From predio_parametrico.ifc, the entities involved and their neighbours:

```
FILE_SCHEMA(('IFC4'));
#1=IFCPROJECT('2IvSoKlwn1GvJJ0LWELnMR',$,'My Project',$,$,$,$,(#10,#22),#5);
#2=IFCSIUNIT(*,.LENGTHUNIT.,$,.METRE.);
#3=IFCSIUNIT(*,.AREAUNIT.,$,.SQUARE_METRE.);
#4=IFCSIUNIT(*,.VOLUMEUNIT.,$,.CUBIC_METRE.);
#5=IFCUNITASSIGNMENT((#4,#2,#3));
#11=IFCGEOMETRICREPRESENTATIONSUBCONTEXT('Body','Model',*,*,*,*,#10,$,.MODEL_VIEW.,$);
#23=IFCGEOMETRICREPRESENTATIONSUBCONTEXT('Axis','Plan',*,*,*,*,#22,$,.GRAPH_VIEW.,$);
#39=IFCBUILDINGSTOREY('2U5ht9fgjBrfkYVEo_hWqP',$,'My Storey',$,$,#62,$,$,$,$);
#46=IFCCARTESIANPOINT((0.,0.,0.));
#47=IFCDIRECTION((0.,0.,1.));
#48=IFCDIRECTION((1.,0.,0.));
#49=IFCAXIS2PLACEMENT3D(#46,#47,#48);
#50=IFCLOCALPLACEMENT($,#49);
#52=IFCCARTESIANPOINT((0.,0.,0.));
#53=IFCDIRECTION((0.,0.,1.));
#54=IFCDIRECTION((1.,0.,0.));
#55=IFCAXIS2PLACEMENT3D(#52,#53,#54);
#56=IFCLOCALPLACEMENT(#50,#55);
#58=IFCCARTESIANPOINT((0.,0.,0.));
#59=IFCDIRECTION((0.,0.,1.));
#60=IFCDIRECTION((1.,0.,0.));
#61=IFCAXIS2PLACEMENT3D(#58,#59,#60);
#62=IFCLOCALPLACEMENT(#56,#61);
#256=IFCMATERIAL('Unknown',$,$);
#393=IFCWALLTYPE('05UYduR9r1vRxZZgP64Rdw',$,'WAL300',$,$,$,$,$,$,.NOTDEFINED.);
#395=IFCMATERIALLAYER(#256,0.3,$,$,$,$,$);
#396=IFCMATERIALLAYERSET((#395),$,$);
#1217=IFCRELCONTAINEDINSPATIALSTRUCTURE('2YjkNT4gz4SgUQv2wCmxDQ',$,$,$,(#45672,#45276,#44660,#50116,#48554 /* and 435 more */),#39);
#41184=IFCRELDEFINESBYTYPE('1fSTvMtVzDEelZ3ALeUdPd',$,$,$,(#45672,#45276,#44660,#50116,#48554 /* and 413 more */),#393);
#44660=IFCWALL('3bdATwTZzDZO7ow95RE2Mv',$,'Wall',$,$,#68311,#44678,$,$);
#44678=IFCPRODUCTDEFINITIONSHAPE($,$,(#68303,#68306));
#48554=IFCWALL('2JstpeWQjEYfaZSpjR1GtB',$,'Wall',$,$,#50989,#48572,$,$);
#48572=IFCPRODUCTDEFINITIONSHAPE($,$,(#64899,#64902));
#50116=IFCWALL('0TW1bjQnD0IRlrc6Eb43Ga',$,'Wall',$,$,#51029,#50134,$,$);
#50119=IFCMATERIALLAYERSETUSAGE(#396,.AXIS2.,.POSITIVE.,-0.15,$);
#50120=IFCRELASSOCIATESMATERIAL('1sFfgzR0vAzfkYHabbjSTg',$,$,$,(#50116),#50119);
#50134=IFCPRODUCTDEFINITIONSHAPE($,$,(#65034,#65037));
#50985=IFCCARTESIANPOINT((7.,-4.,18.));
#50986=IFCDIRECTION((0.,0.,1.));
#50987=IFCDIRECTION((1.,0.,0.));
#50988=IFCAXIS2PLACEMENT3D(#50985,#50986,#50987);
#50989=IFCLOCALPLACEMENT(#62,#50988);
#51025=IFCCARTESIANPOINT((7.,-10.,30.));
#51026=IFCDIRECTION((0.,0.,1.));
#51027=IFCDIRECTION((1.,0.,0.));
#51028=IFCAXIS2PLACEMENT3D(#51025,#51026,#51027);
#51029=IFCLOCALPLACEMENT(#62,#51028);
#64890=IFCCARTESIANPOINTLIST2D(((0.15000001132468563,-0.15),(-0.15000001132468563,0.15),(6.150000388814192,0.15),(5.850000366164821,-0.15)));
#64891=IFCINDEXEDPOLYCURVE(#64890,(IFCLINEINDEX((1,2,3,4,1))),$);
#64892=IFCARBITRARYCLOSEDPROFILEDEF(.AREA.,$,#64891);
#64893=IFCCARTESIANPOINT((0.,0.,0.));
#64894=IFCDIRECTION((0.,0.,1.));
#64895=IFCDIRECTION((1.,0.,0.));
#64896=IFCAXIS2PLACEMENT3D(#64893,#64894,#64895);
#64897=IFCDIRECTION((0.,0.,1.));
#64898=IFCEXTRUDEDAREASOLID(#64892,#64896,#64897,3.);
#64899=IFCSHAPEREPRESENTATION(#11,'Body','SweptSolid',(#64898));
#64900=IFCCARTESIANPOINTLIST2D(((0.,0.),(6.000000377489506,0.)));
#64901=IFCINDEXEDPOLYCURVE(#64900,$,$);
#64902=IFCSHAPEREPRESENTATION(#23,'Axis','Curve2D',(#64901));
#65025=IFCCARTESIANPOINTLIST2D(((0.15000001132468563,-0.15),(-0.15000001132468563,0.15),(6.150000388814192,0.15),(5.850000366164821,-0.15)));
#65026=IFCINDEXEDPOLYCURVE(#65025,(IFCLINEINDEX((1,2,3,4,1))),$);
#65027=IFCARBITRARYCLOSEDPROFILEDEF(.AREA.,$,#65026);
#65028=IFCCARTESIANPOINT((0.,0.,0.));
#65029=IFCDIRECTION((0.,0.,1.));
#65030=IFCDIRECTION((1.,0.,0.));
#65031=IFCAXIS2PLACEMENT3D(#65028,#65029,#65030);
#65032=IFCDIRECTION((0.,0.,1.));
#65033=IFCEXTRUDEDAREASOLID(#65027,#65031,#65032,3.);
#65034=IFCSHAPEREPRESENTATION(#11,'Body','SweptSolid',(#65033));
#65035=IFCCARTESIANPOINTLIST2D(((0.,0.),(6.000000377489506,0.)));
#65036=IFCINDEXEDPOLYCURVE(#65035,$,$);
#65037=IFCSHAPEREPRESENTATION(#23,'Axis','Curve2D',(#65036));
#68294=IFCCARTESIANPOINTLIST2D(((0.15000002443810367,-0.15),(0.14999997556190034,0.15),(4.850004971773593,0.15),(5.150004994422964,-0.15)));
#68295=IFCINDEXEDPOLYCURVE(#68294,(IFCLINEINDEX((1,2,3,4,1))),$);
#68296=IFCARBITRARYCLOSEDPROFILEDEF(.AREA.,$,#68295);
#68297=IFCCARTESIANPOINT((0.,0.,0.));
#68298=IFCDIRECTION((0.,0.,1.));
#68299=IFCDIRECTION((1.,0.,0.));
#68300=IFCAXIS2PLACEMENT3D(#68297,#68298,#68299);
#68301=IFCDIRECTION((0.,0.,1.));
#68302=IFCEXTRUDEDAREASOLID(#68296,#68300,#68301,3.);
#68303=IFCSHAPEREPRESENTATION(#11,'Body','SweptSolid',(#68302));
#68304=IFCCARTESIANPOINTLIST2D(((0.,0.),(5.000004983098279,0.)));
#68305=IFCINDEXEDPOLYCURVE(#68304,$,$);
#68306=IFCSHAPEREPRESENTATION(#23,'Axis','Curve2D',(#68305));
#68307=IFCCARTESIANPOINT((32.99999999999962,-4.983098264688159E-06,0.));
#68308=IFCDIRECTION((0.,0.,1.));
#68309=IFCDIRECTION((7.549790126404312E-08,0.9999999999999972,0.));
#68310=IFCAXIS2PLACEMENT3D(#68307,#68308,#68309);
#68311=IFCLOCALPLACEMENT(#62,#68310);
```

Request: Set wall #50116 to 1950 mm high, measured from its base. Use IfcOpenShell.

```python
import ifcopenshell
import ifcopenshell.geom
import ifcopenshell.util.representation
import ifcopenshell.util.shape

model = ifcopenshell.open("predio_parametrico.ifc")
settings = ifcopenshell.geom.settings()


def volume(element):
    """Net volume in cubic metres, openings subtracted."""
    shape = ifcopenshell.geom.create_shape(settings, element)
    return ifcopenshell.util.shape.get_volume(shape.geometry)


wall = model.by_guid("0TW1bjQnD0IRlrc6Eb43Ga")
before = volume(wall)

body = ifcopenshell.util.representation.get_representation(wall, "Model", "Body")
solid = body.Items[0]
old_height = solid.Depth
solid.Depth = 1.95
after = volume(wall)

print(f"height {old_height:g} -> {solid.Depth:g}, volume {before:.3f} -> {after:.3f} m3")

model.write("predio_parametrico_rev.ifc")
```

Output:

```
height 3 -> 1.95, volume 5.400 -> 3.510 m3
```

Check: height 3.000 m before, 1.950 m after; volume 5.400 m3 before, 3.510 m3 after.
